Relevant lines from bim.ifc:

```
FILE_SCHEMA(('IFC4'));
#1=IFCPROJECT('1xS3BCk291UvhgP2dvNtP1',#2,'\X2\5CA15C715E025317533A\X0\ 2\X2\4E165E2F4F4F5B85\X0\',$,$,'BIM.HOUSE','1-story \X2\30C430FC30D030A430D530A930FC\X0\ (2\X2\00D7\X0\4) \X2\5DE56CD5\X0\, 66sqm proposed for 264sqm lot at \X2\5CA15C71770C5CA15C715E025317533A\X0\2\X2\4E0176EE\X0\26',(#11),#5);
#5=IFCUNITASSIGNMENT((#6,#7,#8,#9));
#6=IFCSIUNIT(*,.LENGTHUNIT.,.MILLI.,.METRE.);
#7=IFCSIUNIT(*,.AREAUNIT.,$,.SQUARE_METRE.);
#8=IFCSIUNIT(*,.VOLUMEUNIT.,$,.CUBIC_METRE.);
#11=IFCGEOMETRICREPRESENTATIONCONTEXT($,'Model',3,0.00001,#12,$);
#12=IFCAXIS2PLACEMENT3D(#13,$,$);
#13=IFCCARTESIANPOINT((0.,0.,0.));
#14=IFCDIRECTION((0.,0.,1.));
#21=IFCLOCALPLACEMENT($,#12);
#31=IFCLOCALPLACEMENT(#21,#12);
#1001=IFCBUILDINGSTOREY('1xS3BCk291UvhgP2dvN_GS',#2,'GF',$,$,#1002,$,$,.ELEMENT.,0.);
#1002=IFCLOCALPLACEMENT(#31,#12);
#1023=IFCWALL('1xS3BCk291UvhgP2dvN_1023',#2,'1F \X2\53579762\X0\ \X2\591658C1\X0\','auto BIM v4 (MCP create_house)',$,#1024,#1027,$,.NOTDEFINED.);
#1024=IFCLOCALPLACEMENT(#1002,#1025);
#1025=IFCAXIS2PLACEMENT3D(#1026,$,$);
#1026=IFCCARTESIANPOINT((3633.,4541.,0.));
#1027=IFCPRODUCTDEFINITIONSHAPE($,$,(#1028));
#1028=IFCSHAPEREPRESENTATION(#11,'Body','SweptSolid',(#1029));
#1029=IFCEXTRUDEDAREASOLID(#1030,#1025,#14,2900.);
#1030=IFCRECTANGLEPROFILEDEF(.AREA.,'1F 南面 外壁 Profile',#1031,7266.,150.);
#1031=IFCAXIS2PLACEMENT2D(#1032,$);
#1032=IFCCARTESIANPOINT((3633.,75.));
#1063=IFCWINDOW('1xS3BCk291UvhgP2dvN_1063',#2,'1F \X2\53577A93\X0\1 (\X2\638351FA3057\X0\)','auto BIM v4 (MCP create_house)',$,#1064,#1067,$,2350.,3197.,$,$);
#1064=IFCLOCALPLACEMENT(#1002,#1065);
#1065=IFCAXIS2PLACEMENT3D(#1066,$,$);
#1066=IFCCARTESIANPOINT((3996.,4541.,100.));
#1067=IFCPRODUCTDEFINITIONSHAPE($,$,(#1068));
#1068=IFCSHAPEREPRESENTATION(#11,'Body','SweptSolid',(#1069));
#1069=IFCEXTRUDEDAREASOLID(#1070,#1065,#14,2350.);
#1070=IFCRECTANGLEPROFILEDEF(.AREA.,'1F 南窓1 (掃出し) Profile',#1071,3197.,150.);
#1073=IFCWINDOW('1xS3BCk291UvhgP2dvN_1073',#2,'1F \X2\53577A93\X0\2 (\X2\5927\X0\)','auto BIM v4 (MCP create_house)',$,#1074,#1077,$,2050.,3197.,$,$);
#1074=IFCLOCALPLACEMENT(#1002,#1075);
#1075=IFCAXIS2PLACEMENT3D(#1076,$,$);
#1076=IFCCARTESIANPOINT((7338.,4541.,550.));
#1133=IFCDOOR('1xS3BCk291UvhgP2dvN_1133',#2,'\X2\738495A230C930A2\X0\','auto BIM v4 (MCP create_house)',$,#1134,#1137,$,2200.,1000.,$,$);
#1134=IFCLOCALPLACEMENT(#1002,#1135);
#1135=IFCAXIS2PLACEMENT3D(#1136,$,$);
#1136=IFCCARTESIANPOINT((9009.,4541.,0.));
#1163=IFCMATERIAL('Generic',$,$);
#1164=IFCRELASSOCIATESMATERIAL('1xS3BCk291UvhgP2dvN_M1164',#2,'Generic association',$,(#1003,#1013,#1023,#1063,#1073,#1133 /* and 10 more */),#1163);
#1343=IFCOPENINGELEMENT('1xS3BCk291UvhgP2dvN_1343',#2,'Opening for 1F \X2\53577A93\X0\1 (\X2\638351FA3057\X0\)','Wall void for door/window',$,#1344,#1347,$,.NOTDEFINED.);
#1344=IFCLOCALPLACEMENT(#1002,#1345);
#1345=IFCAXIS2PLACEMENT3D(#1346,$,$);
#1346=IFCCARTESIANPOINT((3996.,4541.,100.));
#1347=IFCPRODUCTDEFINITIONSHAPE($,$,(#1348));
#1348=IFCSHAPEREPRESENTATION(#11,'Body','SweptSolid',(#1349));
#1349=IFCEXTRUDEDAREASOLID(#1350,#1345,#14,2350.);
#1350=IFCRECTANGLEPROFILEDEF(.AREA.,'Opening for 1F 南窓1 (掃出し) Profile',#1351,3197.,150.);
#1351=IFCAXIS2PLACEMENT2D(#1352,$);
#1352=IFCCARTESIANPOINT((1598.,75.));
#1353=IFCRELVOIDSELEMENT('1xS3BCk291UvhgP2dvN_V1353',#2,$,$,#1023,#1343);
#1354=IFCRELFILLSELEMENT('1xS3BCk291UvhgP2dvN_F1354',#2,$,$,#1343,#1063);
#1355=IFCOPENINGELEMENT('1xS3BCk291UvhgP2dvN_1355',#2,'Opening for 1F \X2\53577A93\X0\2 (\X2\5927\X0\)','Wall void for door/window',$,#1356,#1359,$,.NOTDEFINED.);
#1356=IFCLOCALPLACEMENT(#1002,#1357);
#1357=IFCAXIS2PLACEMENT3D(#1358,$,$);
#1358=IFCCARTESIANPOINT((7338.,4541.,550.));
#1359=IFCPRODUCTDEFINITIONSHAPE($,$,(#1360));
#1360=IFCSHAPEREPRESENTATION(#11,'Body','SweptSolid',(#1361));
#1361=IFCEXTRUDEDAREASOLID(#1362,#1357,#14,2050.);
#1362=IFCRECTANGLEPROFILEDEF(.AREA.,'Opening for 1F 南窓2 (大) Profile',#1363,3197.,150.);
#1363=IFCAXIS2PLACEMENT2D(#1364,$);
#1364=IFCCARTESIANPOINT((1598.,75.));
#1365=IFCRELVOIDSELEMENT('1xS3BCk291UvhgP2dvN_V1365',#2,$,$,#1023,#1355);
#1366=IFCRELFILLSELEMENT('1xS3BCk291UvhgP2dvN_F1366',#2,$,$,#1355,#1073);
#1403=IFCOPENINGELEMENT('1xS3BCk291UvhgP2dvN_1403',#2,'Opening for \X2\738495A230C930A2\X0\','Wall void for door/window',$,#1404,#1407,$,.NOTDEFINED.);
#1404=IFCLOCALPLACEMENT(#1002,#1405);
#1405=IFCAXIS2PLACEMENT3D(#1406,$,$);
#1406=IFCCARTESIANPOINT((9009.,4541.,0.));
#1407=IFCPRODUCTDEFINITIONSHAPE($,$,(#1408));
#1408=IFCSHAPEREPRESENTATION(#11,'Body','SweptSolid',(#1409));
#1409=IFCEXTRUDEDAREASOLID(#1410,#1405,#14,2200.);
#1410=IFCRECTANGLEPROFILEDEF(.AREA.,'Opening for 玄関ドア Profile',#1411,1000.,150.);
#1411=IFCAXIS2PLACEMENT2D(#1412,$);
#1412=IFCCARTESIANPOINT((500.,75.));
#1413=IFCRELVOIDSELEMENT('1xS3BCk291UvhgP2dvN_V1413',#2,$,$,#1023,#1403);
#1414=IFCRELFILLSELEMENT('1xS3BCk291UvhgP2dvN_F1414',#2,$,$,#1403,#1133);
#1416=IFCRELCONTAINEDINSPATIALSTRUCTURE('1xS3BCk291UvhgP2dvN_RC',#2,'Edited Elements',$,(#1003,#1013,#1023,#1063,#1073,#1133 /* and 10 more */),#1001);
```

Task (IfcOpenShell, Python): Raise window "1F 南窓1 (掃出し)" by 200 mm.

```python
import numpy as np
import ifcopenshell
import ifcopenshell.api.geometry
import ifcopenshell.util.placement
import ifcopenshell.util.unit

model = ifcopenshell.open("bim.ifc")
unit_scale = ifcopenshell.util.unit.calculate_unit_scale(model)

window = model.by_guid("1xS3BCk291UvhgP2dvN_1063")
opening = window.FillsVoids[0].RelatingOpeningElement
dz = 0.2 / unit_scale

shift = np.array([0.0, 0.0, dz])
# The window is not placed relative to its opening, so move both.
for product in (opening, window):
    matrix = ifcopenshell.util.placement.get_local_placement(product.ObjectPlacement)
    matrix[:3, 3] += shift
    ifcopenshell.api.geometry.edit_object_placement(model, product=product, matrix=matrix, is_si=False)

print(f"moved by {dz * unit_scale:+.3f} m")

model.write("bim-out.ifc")
```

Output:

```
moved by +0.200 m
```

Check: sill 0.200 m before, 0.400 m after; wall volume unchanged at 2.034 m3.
